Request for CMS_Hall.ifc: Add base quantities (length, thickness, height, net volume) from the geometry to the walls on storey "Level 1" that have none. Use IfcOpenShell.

First a look at what the model holds.

```python
import ifcopenshell
import ifcopenshell.util.element
import ifcopenshell.util.unit

model = ifcopenshell.open("CMS_Hall.ifc")
print(model.schema)
for unit_type in ("LENGTHUNIT", "AREAUNIT", "VOLUMEUNIT"):
    print(unit_type, ifcopenshell.util.unit.calculate_unit_scale(model, unit_type))
storey = next(s for s in model.by_type("IfcBuildingStorey") if s.Name == "Level 1")
walls = [e for e in ifcopenshell.util.element.get_decomposition(storey) if e.is_a("IfcWall")]
for e in sorted(walls, key=lambda e: e.id()):
    print(e.id(), e.is_a(), e.Name, list(ifcopenshell.util.element.get_psets(e, qtos_only=True)), sep=" | ")
```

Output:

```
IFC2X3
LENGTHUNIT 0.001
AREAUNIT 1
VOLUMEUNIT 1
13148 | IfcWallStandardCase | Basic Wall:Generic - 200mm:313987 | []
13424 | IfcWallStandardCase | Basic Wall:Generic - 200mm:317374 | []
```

```python
import ifcopenshell
import ifcopenshell.api.pset
import ifcopenshell.geom
import ifcopenshell.util.element
import ifcopenshell.util.shape
import ifcopenshell.util.unit

model = ifcopenshell.open("CMS_Hall.ifc")
unit_scale = ifcopenshell.util.unit.calculate_unit_scale(model)
volume_scale = ifcopenshell.util.unit.calculate_unit_scale(model, "VOLUMEUNIT")
settings = ifcopenshell.geom.settings()

storey = next(s for s in model.by_type("IfcBuildingStorey") if s.Name == "Level 1")
walls = [e for e in ifcopenshell.util.element.get_decomposition(storey) if e.is_a("IfcWall")]

for e in sorted(walls, key=lambda e: e.id()):
    if ifcopenshell.util.element.get_psets(e, qtos_only=True, should_inherit=False):
        continue
    # Geometry comes back in metres, in the element's own axes.
    shape = ifcopenshell.geom.create_shape(settings, e)
    values = {
        "Length": ifcopenshell.util.shape.get_x(shape.geometry) / unit_scale,
        "Width": ifcopenshell.util.shape.get_y(shape.geometry) / unit_scale,
        "Height": ifcopenshell.util.shape.get_z(shape.geometry) / unit_scale,
        "NetVolume": ifcopenshell.util.shape.get_volume(shape.geometry) / volume_scale,
    }
    qto = ifcopenshell.api.pset.add_qto(model, product=e, name="BaseQuantities")
    ifcopenshell.api.pset.edit_qto(model, qto=qto, properties=values)
    print(e.id(), {k: round(v, 3) for k, v in values.items()})

model.write("CMS_Hall_v2.ifc")
```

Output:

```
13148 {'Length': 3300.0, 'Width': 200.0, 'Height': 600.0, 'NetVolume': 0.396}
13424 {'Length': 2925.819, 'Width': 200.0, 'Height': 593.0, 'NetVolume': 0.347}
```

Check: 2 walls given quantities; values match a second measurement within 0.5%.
